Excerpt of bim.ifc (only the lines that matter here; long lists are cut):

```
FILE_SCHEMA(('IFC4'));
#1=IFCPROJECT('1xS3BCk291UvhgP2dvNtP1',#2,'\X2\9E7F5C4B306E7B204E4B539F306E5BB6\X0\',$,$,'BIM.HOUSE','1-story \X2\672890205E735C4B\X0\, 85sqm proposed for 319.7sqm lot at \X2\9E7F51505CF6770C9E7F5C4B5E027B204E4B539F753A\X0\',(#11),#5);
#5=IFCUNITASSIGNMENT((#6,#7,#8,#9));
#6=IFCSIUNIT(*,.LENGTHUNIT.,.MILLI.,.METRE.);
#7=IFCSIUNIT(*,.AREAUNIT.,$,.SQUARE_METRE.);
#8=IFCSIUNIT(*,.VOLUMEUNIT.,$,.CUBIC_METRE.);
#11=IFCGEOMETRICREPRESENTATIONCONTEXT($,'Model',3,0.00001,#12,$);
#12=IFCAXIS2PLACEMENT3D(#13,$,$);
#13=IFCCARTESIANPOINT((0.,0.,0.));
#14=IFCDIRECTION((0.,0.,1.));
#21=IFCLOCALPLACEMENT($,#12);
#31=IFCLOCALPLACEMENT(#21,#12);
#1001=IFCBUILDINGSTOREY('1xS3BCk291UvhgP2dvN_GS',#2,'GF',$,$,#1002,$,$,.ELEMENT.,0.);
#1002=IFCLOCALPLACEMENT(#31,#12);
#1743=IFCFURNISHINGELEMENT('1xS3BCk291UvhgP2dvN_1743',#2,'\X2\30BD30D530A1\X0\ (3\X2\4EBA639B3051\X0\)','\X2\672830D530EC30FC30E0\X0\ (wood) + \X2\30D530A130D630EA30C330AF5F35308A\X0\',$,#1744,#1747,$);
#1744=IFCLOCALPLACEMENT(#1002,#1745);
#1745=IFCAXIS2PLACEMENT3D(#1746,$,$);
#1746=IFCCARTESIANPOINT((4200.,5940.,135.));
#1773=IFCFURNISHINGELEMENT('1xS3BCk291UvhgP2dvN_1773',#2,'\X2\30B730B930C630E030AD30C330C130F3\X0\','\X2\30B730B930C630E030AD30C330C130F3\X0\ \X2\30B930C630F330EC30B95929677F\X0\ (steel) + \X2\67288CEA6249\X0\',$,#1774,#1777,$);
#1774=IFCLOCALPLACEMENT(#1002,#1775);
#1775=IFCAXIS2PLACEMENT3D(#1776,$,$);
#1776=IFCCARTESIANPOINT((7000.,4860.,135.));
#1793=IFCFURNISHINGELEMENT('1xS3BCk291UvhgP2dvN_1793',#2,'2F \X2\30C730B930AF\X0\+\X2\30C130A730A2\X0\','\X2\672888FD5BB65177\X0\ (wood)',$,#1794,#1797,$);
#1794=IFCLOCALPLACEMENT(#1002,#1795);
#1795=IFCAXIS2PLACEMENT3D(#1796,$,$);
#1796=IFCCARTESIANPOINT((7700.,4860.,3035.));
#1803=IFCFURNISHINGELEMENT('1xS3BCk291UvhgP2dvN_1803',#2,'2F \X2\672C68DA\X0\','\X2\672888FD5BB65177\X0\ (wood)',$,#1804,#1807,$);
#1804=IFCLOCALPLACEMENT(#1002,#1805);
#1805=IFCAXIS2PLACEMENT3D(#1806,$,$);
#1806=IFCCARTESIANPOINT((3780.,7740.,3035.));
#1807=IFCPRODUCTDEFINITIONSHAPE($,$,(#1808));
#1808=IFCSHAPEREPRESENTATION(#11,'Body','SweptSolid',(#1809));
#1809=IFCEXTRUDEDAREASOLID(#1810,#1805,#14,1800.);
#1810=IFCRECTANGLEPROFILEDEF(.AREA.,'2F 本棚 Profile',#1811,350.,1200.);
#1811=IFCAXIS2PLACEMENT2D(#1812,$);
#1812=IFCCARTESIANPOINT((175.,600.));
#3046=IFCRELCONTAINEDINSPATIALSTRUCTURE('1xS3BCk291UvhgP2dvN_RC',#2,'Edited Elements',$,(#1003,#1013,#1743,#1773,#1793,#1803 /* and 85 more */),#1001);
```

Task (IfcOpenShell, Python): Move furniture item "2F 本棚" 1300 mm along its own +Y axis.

```python
import ifcopenshell
import ifcopenshell.api.geometry
import ifcopenshell.util.placement
import ifcopenshell.util.unit

model = ifcopenshell.open("bim.ifc")
unit_scale = ifcopenshell.util.unit.calculate_unit_scale(model)

item = model.by_guid("1xS3BCk291UvhgP2dvN_1803")
matrix = ifcopenshell.util.placement.get_local_placement(item.ObjectPlacement)
matrix[:3, 3] += matrix[:3, 1] * 1.3 / unit_scale
ifcopenshell.api.geometry.edit_object_placement(model, product=item, matrix=matrix, is_si=False)

print(ifcopenshell.util.placement.get_local_placement(item.ObjectPlacement).round(3) + 0.0)

model.write("bim_v2.ifc")
```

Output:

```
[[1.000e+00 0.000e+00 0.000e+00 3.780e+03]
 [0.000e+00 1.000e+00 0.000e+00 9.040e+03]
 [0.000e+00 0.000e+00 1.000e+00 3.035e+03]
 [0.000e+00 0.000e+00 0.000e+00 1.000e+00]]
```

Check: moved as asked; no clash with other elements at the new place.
